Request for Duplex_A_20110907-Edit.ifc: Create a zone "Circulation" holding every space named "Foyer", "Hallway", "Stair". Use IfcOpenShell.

First a look at what the model holds.

```python
import ifcopenshell

model = ifcopenshell.open("Duplex_A_20110907-Edit.ifc")
print(model.schema)
seen = {}
for space in model.by_type("IfcSpace"):
    seen[space.LongName] = seen.get(space.LongName, 0) + 1
for name, count in sorted(seen.items(), key=str):
    print(count, "x", name)
print("zones:", [z.Name for z in model.by_type("IfcZone")][:20])
```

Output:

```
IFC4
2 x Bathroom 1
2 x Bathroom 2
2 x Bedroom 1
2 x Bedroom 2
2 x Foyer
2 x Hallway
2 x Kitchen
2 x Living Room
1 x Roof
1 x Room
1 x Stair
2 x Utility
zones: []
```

```python
import ifcopenshell
import ifcopenshell.api.group
import ifcopenshell.api.root

model = ifcopenshell.open("Duplex_A_20110907-Edit.ifc")

names = {"Foyer", "Hallway", "Stair"}
spaces = [s for s in model.by_type("IfcSpace") if s.LongName in names]

zone = ifcopenshell.api.root.create_entity(model, ifc_class="IfcZone", name="Circulation")
ifcopenshell.api.group.assign_group(model, products=spaces, group=zone)
print(len(spaces), "spaces in", zone.Name)

model.write("Duplex_A_20110907-Edit-out.ifc")
```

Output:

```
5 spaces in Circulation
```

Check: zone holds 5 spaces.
